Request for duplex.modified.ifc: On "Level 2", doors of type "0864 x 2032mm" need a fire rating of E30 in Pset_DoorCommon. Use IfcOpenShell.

First a look at what the model holds.

```python
import ifcopenshell
import ifcopenshell.util.element

model = ifcopenshell.open("duplex.modified.ifc")
print(model.schema)
storey = next(s for s in model.by_type("IfcBuildingStorey") if s.Name == "Level 2")
doors = [e for e in ifcopenshell.util.element.get_decomposition(storey) if e.is_a("IfcDoor")]
seen = {}
for e in doors:
    element_type = ifcopenshell.util.element.get_type(e)
    key = (element_type.Name if element_type != e and element_type else None, ifcopenshell.util.element.get_pset(e, "Pset_DoorCommon", "FireRating"))
    seen[key] = seen.get(key, 0) + 1
for (name, value), count in sorted(seen.items(), key=str):
    print(count, "x", name, "|", value)
```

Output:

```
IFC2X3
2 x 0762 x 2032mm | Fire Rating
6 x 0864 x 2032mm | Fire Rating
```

```python
import ifcopenshell
import ifcopenshell.api.pset
import ifcopenshell.util.element

model = ifcopenshell.open("duplex.modified.ifc")

storey = next(s for s in model.by_type("IfcBuildingStorey") if s.Name == "Level 2")
doors = [e for e in ifcopenshell.util.element.get_decomposition(storey) if e.is_a("IfcDoor")]

count = 0
for e in doors:
    element_type = ifcopenshell.util.element.get_type(e)
    if element_type in (None, e) or element_type.Name != "0864 x 2032mm":
        continue
    # add_pset returns the element's existing set when there is one.
    pset = ifcopenshell.api.pset.add_pset(model, product=e, name="Pset_DoorCommon")
    ifcopenshell.api.pset.edit_pset(model, pset=pset, properties={"FireRating": "E30"})
    count += 1

print(count, "doors updated")

model.write("duplex.modified_edited.ifc")
```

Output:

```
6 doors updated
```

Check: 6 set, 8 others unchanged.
